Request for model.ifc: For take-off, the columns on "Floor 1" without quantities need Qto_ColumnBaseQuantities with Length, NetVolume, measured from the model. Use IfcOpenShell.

First a look at what the model holds.

```python
import ifcopenshell
import ifcopenshell.util.element
import ifcopenshell.util.unit

model = ifcopenshell.open("model.ifc")
print(model.schema)
for unit_type in ("LENGTHUNIT", "AREAUNIT", "VOLUMEUNIT"):
    print(unit_type, ifcopenshell.util.unit.calculate_unit_scale(model, unit_type))
storey = next(s for s in model.by_type("IfcBuildingStorey") if s.Name == "Floor 1")
columns = [e for e in ifcopenshell.util.element.get_decomposition(storey) if e.is_a("IfcColumn")]
for e in sorted(columns, key=lambda e: e.id()):
    print(e.id(), e.is_a(), e.Name, list(ifcopenshell.util.element.get_psets(e, qtos_only=True)), sep=" | ")
```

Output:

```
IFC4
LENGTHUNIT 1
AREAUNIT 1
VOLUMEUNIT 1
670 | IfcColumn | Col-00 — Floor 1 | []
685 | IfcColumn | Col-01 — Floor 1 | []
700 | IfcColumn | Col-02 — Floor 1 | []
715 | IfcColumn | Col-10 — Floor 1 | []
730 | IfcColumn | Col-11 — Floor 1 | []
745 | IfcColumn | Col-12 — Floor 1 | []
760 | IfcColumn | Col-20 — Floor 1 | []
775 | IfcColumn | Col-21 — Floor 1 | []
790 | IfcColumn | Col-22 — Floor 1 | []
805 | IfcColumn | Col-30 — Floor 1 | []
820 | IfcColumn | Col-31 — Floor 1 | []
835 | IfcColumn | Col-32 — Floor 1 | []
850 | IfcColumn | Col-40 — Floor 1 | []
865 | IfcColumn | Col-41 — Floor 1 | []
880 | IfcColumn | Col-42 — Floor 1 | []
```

```python
import ifcopenshell
import ifcopenshell.api.pset
import ifcopenshell.geom
import ifcopenshell.util.element
import ifcopenshell.util.shape
import ifcopenshell.util.unit

model = ifcopenshell.open("model.ifc")
unit_scale = ifcopenshell.util.unit.calculate_unit_scale(model)
volume_scale = ifcopenshell.util.unit.calculate_unit_scale(model, "VOLUMEUNIT")
settings = ifcopenshell.geom.settings()

storey = next(s for s in model.by_type("IfcBuildingStorey") if s.Name == "Floor 1")
columns = [e for e in ifcopenshell.util.element.get_decomposition(storey) if e.is_a("IfcColumn")]

for e in sorted(columns, key=lambda e: e.id()):
    if ifcopenshell.util.element.get_psets(e, qtos_only=True, should_inherit=False):
        continue
    # Geometry comes back in metres, in the element's own axes.
    shape = ifcopenshell.geom.create_shape(settings, e)
    values = {
        "Length": ifcopenshell.util.shape.get_z(shape.geometry) / unit_scale,
        "NetVolume": ifcopenshell.util.shape.get_volume(shape.geometry) / volume_scale,
    }
    qto = ifcopenshell.api.pset.add_qto(model, product=e, name="Qto_ColumnBaseQuantities")
    ifcopenshell.api.pset.edit_qto(model, qto=qto, properties=values)
    print(e.id(), {k: round(v, 3) for k, v in values.items()})

model.write("model-out.ifc")
```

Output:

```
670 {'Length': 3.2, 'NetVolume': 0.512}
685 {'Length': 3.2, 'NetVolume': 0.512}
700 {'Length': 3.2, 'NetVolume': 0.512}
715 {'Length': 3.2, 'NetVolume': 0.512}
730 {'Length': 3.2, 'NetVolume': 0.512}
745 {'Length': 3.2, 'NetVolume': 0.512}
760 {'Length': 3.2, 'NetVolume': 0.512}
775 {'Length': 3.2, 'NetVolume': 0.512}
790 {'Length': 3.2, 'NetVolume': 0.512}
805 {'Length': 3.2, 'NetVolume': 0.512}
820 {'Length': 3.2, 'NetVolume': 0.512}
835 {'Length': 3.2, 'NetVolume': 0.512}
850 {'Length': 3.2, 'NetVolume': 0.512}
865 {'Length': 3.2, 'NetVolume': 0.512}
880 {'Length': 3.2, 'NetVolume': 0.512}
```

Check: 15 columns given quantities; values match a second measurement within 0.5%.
